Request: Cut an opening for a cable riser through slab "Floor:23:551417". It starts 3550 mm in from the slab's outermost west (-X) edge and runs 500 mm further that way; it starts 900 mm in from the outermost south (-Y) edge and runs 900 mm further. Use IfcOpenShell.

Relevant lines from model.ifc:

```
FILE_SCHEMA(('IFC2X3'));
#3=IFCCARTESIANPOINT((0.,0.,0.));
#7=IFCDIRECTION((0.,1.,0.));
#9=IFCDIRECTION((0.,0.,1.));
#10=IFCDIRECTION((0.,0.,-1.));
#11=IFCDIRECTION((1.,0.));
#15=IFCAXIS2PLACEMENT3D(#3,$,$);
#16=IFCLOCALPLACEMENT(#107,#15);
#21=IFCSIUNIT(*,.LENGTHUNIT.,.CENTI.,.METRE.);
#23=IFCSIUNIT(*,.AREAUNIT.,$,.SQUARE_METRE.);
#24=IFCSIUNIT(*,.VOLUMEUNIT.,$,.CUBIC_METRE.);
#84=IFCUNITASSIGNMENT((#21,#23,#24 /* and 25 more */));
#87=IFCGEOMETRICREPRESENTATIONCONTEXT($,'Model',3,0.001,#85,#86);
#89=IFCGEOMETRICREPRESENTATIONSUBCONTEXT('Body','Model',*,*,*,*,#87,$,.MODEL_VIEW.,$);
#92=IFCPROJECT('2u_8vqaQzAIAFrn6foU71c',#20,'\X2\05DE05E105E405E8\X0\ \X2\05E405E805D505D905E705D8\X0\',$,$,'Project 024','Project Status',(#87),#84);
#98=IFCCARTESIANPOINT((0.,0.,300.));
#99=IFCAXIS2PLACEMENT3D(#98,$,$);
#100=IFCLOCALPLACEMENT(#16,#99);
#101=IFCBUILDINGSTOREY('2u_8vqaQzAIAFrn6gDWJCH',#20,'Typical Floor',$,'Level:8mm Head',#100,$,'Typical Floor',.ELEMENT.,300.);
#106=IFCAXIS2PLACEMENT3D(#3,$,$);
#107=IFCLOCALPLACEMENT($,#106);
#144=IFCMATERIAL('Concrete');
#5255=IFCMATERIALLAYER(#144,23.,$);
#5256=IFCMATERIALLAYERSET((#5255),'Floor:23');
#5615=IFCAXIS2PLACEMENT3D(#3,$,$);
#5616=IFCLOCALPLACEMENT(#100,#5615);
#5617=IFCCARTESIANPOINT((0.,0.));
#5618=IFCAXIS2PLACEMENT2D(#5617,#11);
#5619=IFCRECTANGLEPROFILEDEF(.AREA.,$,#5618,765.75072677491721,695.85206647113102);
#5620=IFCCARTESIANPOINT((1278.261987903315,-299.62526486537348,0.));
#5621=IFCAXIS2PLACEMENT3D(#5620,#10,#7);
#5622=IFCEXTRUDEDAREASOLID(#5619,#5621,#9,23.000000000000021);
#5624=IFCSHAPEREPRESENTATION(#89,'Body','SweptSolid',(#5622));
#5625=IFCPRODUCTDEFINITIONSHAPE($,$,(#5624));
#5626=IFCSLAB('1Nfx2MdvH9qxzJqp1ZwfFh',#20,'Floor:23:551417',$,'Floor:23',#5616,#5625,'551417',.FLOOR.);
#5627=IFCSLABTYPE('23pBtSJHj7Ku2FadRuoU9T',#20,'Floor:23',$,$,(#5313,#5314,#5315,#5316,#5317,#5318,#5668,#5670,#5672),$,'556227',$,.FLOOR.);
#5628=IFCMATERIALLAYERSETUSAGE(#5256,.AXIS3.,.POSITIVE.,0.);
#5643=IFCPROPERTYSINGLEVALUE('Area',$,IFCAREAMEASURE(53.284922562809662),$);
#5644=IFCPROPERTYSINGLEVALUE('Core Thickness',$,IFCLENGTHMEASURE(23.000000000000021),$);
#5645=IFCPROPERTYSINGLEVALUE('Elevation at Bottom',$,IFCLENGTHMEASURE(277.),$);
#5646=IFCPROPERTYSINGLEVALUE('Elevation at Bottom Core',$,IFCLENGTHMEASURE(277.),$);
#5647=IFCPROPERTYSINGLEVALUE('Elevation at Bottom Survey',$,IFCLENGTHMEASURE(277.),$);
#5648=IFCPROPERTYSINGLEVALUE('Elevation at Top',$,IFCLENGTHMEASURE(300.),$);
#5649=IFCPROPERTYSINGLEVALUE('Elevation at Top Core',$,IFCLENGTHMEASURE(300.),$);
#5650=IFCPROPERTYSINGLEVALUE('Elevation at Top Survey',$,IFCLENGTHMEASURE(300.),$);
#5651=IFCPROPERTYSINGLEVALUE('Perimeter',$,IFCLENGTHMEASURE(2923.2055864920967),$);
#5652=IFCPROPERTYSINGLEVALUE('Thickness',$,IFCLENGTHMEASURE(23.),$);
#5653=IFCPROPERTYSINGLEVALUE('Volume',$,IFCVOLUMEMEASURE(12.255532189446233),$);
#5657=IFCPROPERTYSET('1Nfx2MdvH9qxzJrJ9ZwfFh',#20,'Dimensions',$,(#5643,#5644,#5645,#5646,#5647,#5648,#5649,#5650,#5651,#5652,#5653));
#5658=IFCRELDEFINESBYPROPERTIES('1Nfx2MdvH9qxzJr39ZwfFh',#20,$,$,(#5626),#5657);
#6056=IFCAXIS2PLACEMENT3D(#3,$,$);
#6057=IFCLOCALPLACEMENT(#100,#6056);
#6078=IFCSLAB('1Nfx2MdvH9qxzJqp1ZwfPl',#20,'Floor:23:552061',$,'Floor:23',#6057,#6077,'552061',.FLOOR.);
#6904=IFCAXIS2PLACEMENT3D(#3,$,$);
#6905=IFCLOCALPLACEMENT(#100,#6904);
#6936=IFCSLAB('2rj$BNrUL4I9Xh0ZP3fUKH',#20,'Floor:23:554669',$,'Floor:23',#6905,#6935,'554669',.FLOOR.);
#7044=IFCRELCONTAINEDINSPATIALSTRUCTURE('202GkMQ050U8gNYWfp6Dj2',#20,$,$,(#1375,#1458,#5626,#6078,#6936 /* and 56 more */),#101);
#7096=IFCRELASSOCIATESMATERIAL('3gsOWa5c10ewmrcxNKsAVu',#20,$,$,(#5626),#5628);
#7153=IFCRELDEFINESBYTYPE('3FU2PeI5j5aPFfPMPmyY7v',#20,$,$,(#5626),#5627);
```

```python
import numpy as np
import ifcopenshell
import ifcopenshell.api.feature
import ifcopenshell.api.geometry
import ifcopenshell.api.pset
import ifcopenshell.api.root
import ifcopenshell.geom
import ifcopenshell.util.element
import ifcopenshell.util.placement
import ifcopenshell.util.representation
import ifcopenshell.util.shape
import ifcopenshell.util.unit

model = ifcopenshell.open("model.ifc")
unit_scale = ifcopenshell.util.unit.calculate_unit_scale(model)
area_scale = ifcopenshell.util.unit.calculate_unit_scale(model, "AREAUNIT")
volume_scale = ifcopenshell.util.unit.calculate_unit_scale(model, "VOLUMEUNIT")
settings = ifcopenshell.geom.settings()


def volume(element):
    """Net volume in cubic metres, openings subtracted."""
    shape = ifcopenshell.geom.create_shape(settings, element)
    return ifcopenshell.util.shape.get_volume(shape.geometry)


slab = model.by_guid("1Nfx2MdvH9qxzJqp1ZwfFh")
before = volume(slab)

# Extent in the slab's own axes, in metres. The edges named are its -X and -Y sides.
slab_shape = ifcopenshell.geom.create_shape(settings, slab)
vertices = ifcopenshell.util.shape.get_vertices(slab_shape.geometry)
x_min, y_min, bottom = vertices.min(axis=0)
top = vertices[:, 2].max()

opening = ifcopenshell.api.root.create_entity(model, ifc_class="IfcOpeningElement", name="Cable riser opening")
context = ifcopenshell.util.representation.get_context(model, "Model", "Body", "MODEL_VIEW")
width, depth = 0.5, 0.9
outline = [(0.0, 0.0), (width, 0.0), (width, depth), (0.0, depth), (0.0, 0.0)]
# Overshoot both faces by 50 mm so the cut is clean.
shape = ifcopenshell.api.geometry.add_slab_representation(
    model, context=context, depth=top - bottom + 0.1, polyline=outline
)
ifcopenshell.api.geometry.assign_representation(model, product=opening, representation=shape)

matrix = ifcopenshell.util.placement.get_local_placement(slab.ObjectPlacement)
matrix[:, 3] = matrix @ np.append(np.array([x_min + 3.55, y_min + 0.9, bottom - 0.05]) / unit_scale, 1.0)
ifcopenshell.api.geometry.edit_object_placement(model, product=opening, matrix=matrix, is_si=False)
ifcopenshell.api.feature.add_feature(model, feature=opening, element=slab)

after = volume(slab)

# Update the slab's stored quantities.
pset = model.by_id(ifcopenshell.util.element.get_pset(slab, "Dimensions", should_inherit=False)["id"])
ifcopenshell.api.pset.edit_pset(model, pset=pset, properties={
    "Area": model.create_entity("IfcAreaMeasure", after / (top - bottom) / area_scale),
    "Volume": model.create_entity("IfcVolumeMeasure", after / volume_scale),
})

print(f"slab volume {before:.3f} -> {after:.3f} m3")

model.write("model_rev.ifc")
```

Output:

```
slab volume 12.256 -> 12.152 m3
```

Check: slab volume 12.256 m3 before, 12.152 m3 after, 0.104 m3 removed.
